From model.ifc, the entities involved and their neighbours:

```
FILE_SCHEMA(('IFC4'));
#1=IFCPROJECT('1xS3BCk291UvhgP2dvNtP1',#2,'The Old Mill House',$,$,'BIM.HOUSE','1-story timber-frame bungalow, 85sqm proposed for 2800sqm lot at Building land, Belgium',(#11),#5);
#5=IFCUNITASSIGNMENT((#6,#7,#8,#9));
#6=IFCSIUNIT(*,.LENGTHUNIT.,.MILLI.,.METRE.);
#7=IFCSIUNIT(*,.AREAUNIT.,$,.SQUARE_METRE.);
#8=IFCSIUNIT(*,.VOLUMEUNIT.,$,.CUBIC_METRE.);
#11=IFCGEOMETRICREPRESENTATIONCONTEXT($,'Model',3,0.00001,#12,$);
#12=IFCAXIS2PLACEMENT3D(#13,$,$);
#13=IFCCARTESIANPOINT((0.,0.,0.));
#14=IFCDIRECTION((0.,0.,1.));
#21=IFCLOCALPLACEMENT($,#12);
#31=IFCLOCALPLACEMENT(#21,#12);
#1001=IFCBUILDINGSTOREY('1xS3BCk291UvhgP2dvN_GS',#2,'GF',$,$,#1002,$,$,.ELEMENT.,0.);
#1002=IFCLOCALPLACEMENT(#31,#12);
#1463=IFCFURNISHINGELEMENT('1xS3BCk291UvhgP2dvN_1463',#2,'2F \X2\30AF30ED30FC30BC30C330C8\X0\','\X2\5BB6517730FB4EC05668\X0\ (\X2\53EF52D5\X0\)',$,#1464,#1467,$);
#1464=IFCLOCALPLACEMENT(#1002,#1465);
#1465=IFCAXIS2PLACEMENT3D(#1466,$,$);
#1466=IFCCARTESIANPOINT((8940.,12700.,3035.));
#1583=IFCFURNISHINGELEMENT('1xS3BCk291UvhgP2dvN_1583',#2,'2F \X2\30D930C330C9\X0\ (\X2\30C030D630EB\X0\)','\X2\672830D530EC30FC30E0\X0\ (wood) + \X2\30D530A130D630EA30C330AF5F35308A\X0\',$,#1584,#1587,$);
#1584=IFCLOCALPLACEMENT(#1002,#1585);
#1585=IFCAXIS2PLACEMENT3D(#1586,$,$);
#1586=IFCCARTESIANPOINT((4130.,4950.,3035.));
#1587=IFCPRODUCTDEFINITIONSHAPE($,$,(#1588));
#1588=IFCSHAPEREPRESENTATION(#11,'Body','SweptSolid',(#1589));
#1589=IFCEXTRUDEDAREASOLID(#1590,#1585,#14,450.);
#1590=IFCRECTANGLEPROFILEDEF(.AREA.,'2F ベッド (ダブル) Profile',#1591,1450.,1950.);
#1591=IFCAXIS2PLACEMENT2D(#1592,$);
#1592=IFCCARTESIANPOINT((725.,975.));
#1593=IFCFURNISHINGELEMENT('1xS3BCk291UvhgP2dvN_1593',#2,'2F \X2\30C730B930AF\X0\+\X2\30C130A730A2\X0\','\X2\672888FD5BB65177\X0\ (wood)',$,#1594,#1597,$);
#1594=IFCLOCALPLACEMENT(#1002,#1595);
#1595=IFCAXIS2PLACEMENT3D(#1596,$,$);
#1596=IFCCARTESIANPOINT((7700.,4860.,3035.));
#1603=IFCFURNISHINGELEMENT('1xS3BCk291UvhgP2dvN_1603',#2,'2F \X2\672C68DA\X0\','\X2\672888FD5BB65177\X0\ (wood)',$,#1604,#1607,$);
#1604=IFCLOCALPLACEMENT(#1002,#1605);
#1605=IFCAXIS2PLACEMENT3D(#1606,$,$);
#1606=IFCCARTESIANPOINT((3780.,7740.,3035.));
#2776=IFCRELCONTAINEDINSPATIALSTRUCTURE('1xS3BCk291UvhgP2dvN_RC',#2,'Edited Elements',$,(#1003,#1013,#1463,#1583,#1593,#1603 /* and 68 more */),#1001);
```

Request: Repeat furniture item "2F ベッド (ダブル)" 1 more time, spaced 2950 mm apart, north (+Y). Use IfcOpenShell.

```python
import numpy as np
import ifcopenshell
import ifcopenshell.api.geometry
import ifcopenshell.api.root
import ifcopenshell.util.element
import ifcopenshell.util.placement
import ifcopenshell.util.unit

model = ifcopenshell.open("model.ifc")
unit_scale = ifcopenshell.util.unit.calculate_unit_scale(model)


def reuse_history(source, copy):
    """copy_class also copies each property set's owner history, people and application; keep the originals."""
    for rel in copy.IsDefinedBy:
        if rel.is_a("IfcRelDefinesByProperties") and (history := rel.RelatingPropertyDefinition.OwnerHistory):
            rel.RelatingPropertyDefinition.OwnerHistory = source.OwnerHistory
            ifcopenshell.util.element.remove_deep2(model, history)


source = model.by_id(1583)
base = ifcopenshell.util.placement.get_local_placement(source.ObjectPlacement)
step = np.array([0.0, 1.0, 0.0]) * 2.95 / unit_scale

for i in range(1, 2):
    copy = ifcopenshell.api.root.copy_class(model, product=source)
    copy.Representation = ifcopenshell.util.element.copy_deep(
        model, source.Representation, exclude=["IfcGeometricRepresentationContext", "IfcRepresentationMap"]
    )
    reuse_history(source, copy)
    matrix = base.copy()
    matrix[:3, 3] += i * step
    print("added at", matrix[:3, 3].round(3) + 0.0)
    ifcopenshell.api.geometry.edit_object_placement(model, product=copy, matrix=matrix, is_si=False)

model.write("model-out.ifc")
```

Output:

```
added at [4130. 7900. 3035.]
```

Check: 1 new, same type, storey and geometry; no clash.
